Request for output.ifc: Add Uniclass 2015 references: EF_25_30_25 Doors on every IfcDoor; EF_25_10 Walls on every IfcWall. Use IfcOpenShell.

First a look at what the model holds.

```python
import ifcopenshell

model = ifcopenshell.open("output.ifc")
print(model.schema)
print("classifications:", [c.Name for c in model.by_type("IfcClassification")])
for ifc_class in ("IfcDoor", "IfcRoof", "IfcStair", "IfcWall", "IfcWindow"):
    print(ifc_class, len(model.by_type(ifc_class)))
```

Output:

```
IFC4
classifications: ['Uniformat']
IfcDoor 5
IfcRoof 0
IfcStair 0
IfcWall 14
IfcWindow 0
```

```python
import ifcopenshell
import ifcopenshell.api.classification

model = ifcopenshell.open("output.ifc")

system = ifcopenshell.api.classification.add_classification(model, classification="Uniclass 2015")

codes = {
    "IfcDoor": ("EF_25_30_25", "Doors"),
    "IfcWall": ("EF_25_10", "Walls"),
}
for ifc_class, (code, name) in codes.items():
    products = model.by_type(ifc_class)
    ifcopenshell.api.classification.add_reference(
        model, products=products, classification=system, identification=code, name=name
    )
    print(code, len(products))

model.write("output_updated.ifc")
```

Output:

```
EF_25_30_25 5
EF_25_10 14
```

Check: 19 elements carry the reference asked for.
